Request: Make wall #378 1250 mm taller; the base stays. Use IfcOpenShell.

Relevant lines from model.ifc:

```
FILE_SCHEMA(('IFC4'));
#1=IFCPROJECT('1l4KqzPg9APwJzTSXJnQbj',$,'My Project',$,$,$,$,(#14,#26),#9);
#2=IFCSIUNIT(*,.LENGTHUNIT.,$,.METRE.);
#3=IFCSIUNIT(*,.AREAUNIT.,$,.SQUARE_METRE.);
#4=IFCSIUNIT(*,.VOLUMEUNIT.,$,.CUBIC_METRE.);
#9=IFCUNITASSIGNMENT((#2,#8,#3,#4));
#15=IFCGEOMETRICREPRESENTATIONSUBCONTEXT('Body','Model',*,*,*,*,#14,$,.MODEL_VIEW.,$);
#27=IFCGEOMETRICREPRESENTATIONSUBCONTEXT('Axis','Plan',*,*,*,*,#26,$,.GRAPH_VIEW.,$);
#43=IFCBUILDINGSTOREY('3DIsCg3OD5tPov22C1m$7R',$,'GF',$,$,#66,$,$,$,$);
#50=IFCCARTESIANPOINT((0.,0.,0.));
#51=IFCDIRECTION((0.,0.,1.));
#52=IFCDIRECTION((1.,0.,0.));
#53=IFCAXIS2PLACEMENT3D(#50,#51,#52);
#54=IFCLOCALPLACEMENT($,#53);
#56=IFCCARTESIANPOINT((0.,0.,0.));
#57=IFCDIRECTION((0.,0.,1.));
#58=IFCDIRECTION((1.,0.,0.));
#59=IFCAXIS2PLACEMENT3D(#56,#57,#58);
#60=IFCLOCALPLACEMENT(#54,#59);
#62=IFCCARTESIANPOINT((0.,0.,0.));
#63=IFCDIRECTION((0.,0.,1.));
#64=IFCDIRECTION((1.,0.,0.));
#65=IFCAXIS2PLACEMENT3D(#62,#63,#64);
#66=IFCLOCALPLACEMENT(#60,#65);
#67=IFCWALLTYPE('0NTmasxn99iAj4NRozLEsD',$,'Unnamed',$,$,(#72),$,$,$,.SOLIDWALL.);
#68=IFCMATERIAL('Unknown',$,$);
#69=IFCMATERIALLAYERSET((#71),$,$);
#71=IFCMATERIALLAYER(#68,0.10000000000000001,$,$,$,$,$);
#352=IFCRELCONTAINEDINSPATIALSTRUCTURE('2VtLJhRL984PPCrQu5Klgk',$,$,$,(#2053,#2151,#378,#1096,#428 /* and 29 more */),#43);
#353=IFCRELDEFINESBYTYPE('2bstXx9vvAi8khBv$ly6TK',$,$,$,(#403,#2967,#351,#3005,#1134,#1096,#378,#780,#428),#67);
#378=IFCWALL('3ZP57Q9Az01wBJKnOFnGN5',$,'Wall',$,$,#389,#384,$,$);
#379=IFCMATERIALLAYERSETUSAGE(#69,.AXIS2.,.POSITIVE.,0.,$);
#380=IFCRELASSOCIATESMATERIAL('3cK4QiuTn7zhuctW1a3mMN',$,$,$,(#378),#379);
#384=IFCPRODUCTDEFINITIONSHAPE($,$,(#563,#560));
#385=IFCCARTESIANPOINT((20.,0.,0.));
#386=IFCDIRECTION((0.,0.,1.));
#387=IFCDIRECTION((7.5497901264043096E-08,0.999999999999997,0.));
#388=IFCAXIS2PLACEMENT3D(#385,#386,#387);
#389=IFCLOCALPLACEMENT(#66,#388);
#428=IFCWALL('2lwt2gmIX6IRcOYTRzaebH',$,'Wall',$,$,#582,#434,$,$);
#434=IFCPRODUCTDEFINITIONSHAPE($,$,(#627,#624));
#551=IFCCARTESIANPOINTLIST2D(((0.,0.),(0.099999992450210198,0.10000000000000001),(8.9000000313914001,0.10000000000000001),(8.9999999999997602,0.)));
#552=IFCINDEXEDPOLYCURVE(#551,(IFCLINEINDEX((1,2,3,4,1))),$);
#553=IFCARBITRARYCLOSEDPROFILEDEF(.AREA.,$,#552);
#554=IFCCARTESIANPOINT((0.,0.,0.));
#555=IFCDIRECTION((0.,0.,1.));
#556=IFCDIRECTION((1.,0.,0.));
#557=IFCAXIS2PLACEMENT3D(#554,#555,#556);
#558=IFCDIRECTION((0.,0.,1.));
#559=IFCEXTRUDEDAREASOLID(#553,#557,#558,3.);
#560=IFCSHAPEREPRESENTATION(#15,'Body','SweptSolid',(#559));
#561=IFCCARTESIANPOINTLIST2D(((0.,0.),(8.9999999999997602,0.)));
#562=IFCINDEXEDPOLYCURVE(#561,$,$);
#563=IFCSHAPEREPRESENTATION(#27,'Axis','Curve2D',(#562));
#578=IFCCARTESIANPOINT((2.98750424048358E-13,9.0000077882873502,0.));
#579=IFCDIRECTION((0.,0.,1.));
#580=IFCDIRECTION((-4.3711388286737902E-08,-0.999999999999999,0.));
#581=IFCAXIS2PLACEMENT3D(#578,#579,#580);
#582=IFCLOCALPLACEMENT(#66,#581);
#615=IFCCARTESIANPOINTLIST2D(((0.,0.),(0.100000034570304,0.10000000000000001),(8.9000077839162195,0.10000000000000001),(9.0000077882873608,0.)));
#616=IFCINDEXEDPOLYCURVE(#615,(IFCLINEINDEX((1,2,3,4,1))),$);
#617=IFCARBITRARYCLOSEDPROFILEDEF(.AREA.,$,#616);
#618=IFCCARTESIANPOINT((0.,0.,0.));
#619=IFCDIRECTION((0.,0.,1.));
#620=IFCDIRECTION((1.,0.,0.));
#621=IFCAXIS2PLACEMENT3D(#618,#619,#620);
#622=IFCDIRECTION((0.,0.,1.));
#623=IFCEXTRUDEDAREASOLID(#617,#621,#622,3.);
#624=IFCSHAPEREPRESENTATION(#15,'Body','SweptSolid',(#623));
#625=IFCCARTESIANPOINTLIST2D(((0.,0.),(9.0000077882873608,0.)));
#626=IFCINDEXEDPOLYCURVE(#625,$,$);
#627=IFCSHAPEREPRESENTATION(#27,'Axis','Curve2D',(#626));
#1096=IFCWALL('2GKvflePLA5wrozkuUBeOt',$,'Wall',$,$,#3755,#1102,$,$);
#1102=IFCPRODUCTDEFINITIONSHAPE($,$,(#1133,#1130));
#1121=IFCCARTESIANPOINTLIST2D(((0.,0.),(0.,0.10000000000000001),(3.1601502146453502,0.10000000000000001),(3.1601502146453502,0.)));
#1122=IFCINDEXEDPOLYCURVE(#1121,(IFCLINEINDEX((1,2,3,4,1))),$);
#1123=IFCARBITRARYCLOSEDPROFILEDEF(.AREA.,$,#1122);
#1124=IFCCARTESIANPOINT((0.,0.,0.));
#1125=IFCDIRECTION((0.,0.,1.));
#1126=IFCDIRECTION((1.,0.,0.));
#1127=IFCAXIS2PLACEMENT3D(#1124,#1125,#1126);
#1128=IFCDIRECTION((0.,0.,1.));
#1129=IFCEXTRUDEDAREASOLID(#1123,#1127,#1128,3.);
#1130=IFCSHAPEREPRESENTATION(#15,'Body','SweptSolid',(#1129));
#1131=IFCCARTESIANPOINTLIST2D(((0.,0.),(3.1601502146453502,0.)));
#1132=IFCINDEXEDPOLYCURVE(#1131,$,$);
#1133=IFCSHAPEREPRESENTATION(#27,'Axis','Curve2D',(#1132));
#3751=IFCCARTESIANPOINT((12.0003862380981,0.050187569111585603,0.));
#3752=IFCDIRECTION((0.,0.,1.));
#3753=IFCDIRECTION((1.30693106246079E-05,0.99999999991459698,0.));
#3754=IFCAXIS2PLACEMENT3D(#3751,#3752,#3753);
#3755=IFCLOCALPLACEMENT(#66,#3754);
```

```python
import ifcopenshell
import ifcopenshell.geom
import ifcopenshell.util.representation
import ifcopenshell.util.shape

model = ifcopenshell.open("model.ifc")
settings = ifcopenshell.geom.settings()


def volume(element):
    """Net volume in cubic metres, openings subtracted."""
    shape = ifcopenshell.geom.create_shape(settings, element)
    return ifcopenshell.util.shape.get_volume(shape.geometry)


wall = model.by_guid("3ZP57Q9Az01wBJKnOFnGN5")
before = volume(wall)

body = ifcopenshell.util.representation.get_representation(wall, "Model", "Body")
solid = body.Items[0]
old_height = solid.Depth
solid.Depth += 1.25
after = volume(wall)

print(f"height {old_height:g} -> {solid.Depth:g}, volume {before:.3f} -> {after:.3f} m3")

model.write("model_updated.ifc")
```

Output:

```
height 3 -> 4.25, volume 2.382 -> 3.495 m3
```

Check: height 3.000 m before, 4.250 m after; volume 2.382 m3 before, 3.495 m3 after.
